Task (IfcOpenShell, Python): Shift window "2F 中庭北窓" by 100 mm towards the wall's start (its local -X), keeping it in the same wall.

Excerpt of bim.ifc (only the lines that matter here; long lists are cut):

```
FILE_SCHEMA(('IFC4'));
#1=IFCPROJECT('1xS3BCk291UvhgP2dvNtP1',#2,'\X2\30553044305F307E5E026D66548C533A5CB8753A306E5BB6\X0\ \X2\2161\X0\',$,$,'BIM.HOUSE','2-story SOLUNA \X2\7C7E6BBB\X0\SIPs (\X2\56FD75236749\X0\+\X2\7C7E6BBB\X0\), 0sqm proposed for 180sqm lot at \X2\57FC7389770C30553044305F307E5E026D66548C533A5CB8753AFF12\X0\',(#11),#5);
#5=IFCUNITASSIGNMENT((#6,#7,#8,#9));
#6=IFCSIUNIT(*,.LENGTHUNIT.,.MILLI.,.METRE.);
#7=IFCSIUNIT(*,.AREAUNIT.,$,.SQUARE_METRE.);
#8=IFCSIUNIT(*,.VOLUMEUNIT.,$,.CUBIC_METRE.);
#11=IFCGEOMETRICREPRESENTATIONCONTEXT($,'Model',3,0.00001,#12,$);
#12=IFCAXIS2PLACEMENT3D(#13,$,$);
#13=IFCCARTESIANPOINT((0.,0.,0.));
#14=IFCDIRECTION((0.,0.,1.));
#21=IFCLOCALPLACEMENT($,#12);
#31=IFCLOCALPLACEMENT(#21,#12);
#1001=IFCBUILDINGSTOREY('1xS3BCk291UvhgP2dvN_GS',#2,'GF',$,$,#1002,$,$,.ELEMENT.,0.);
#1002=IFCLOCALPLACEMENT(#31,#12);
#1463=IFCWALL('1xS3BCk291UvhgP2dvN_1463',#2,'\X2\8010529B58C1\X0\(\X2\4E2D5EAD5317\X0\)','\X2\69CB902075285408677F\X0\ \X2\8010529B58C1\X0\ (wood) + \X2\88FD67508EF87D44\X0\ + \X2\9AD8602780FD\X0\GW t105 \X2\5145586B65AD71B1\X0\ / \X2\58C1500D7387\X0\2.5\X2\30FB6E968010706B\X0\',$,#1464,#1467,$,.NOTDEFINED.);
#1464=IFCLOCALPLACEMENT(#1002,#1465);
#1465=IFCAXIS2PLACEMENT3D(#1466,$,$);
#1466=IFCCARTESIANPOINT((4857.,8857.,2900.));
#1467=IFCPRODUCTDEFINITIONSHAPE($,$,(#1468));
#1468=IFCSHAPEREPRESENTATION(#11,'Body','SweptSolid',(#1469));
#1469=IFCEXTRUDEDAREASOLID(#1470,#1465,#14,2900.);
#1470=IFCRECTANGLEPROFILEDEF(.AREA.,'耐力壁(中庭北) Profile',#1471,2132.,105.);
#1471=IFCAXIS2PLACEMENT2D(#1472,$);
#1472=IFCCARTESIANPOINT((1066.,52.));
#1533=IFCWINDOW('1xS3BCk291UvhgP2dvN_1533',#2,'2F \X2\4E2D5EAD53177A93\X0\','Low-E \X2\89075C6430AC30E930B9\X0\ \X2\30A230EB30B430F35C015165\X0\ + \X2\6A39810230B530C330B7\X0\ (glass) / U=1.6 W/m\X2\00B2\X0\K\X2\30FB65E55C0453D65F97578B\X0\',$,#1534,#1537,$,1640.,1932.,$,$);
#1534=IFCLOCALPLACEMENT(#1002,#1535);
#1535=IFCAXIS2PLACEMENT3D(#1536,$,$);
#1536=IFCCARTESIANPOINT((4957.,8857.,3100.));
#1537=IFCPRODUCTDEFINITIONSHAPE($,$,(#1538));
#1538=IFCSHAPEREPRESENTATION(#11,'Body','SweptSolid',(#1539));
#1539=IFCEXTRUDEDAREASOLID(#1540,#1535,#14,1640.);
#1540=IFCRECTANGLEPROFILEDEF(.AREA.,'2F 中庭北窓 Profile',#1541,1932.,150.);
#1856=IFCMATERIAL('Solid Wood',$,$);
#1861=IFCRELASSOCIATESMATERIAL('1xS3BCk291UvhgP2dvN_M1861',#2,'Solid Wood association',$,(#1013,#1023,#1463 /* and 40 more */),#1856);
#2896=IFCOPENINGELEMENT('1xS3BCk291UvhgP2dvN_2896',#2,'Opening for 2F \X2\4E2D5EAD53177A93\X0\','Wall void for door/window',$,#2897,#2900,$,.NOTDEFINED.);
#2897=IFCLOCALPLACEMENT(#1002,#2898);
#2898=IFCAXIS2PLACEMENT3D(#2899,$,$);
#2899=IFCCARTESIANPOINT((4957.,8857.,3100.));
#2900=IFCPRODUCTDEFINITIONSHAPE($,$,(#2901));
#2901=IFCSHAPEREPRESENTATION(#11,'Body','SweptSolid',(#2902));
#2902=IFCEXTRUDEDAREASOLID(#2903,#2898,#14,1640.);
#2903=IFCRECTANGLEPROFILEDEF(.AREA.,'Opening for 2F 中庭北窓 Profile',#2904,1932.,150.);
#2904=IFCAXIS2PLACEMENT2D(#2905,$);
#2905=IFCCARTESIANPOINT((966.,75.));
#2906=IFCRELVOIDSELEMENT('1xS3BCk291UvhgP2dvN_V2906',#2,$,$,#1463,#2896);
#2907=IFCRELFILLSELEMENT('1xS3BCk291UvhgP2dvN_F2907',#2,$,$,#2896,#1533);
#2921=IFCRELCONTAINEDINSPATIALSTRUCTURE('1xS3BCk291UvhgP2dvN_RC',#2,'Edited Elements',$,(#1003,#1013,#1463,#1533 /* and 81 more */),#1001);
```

```python
import ifcopenshell
import ifcopenshell.api.geometry
import ifcopenshell.util.placement
import ifcopenshell.util.unit

model = ifcopenshell.open("bim.ifc")
unit_scale = ifcopenshell.util.unit.calculate_unit_scale(model)

window = model.by_guid("1xS3BCk291UvhgP2dvN_1533")
opening = window.FillsVoids[0].RelatingOpeningElement
wall = opening.VoidsElements[0].RelatingBuildingElement

wall_matrix = ifcopenshell.util.placement.get_local_placement(wall.ObjectPlacement)
shift = wall_matrix[:3, 0] * -0.1 / unit_scale
before = ifcopenshell.util.placement.get_local_placement(window.ObjectPlacement)[:3, 3].copy()

# The window is not placed relative to its opening, so move both.
for product in (opening, window):
    matrix = ifcopenshell.util.placement.get_local_placement(product.ObjectPlacement)
    matrix[:3, 3] += shift
    ifcopenshell.api.geometry.edit_object_placement(model, product=product, matrix=matrix, is_si=False)

after = ifcopenshell.util.placement.get_local_placement(window.ObjectPlacement)[:3, 3]
print("window moved by", (after - before).round(3) + 0.0)

model.write("bim_updated.ifc")
```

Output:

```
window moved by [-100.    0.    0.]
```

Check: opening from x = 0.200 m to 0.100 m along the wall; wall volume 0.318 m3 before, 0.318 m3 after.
